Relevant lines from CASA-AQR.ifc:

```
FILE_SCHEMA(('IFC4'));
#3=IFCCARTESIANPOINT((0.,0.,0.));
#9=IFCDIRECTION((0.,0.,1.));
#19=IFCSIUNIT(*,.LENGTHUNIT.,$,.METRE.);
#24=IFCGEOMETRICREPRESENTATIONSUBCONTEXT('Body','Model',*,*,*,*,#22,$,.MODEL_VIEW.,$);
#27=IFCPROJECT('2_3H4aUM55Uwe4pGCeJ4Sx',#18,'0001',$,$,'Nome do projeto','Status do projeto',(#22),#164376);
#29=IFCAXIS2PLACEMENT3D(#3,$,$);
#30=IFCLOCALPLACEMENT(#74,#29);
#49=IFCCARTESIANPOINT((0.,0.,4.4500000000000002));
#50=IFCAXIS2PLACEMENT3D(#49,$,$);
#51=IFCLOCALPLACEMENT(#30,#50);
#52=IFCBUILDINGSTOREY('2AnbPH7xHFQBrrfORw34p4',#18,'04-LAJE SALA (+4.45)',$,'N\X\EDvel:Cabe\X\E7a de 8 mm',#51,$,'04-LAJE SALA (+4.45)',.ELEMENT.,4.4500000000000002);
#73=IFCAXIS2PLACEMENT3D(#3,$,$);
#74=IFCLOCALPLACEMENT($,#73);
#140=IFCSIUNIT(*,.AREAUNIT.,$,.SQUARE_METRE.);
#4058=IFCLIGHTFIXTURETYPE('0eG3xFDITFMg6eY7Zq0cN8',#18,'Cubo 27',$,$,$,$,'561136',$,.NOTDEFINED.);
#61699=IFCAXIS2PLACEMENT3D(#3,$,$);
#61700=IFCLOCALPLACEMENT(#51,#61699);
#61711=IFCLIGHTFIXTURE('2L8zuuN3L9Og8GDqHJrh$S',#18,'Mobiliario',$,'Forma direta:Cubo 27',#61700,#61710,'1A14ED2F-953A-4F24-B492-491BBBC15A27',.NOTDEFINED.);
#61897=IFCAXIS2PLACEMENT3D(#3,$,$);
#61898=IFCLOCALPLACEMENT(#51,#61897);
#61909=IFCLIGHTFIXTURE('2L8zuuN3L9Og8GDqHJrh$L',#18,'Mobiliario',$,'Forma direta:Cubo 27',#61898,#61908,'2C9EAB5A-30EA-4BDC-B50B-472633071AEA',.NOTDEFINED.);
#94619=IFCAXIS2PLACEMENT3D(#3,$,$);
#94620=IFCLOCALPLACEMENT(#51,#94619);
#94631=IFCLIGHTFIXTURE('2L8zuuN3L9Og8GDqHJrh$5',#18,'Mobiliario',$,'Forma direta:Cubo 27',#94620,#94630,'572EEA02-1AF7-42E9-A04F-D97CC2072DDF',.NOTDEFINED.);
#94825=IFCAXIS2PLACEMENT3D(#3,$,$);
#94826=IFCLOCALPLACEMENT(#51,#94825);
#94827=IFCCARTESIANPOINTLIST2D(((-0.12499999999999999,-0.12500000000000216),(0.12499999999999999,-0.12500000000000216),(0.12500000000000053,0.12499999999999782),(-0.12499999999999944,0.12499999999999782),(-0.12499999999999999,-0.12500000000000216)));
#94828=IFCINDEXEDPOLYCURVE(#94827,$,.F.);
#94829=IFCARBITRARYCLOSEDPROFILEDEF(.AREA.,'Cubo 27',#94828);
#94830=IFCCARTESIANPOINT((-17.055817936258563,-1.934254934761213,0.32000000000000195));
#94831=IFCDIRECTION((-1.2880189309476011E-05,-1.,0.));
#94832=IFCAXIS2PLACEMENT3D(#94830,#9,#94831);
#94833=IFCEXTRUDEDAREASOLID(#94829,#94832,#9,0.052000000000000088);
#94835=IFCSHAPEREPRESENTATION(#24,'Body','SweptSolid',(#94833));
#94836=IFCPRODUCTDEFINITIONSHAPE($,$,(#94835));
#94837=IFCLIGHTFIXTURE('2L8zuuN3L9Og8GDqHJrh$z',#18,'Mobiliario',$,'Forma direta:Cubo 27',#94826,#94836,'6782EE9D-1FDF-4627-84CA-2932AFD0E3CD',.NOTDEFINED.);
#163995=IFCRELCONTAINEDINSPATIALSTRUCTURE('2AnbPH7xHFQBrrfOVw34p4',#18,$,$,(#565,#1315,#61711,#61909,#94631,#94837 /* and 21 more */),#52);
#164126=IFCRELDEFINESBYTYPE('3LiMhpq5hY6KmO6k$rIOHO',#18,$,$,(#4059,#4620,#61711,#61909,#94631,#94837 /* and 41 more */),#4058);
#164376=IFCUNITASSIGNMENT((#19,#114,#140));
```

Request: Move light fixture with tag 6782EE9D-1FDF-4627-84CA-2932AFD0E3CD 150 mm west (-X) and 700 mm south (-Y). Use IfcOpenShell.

```python
import ifcopenshell
import ifcopenshell.api.geometry
import ifcopenshell.util.placement
import ifcopenshell.util.unit

model = ifcopenshell.open("CASA-AQR.ifc")
unit_scale = ifcopenshell.util.unit.calculate_unit_scale(model)

item = model.by_guid("2L8zuuN3L9Og8GDqHJrh$z")
matrix = ifcopenshell.util.placement.get_local_placement(item.ObjectPlacement)
matrix[0, 3] -= 0.15 / unit_scale
matrix[1, 3] -= 0.7 / unit_scale
ifcopenshell.api.geometry.edit_object_placement(model, product=item, matrix=matrix, is_si=False)

print(ifcopenshell.util.placement.get_local_placement(item.ObjectPlacement).round(3) + 0.0)

model.write("CASA-AQR_edited.ifc")
```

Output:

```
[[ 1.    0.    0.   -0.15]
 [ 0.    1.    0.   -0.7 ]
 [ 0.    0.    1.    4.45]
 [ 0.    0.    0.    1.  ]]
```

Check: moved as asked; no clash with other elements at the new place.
